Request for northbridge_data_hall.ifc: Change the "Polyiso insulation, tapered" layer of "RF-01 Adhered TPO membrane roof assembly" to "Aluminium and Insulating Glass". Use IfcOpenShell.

First a look at what the model holds.

```python
import ifcopenshell
import ifcopenshell.util.element

model = ifcopenshell.open("northbridge_data_hall.ifc")
print(model.schema)
for layer_set in model.by_type("IfcMaterialLayerSet"):
    if layer_set.LayerSetName == "RF-01 Adhered TPO membrane roof assembly":
        for layer in layer_set.MaterialLayers:
            print(layer.id(), layer.Material and layer.Material.Name, layer.LayerThickness, sep=" | ")
        print(len(ifcopenshell.util.element.get_elements_by_material(model, layer_set)), "elements and types use it")
print(sorted(m.Name for m in model.by_type("IfcMaterial") if m.Name)[:60])
```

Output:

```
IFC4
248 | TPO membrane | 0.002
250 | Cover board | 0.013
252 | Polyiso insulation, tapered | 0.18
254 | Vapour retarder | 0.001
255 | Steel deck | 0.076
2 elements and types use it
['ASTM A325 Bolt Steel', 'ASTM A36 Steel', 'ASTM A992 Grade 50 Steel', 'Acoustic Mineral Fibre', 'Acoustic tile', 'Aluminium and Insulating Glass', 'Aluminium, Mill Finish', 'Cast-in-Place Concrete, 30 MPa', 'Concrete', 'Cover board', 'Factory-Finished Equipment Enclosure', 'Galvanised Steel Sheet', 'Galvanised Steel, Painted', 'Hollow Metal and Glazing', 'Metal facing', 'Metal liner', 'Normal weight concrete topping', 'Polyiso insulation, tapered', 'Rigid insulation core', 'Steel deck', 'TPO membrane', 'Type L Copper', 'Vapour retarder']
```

```python
import ifcopenshell
import ifcopenshell.api.material

model = ifcopenshell.open("northbridge_data_hall.ifc")

layer_set = next(s for s in model.by_type("IfcMaterialLayerSet") if s.LayerSetName == "RF-01 Adhered TPO membrane roof assembly")
layer = next(l for l in layer_set.MaterialLayers if l.Material and l.Material.Name == "Polyiso insulation, tapered")
material = next(m for m in model.by_type("IfcMaterial") if m.Name == "Aluminium and Insulating Glass")

# Point this one layer at the other material; renaming the old one would change it everywhere.
ifcopenshell.api.material.edit_layer(model, layer=layer, attributes={"Name": material.Name}, material=material)

print([l.Material.Name if l.Material else None for l in layer_set.MaterialLayers])

model.write("northbridge_data_hall_updated.ifc")
```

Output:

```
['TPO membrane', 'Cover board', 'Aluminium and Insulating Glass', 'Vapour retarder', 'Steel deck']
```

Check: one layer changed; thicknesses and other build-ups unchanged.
